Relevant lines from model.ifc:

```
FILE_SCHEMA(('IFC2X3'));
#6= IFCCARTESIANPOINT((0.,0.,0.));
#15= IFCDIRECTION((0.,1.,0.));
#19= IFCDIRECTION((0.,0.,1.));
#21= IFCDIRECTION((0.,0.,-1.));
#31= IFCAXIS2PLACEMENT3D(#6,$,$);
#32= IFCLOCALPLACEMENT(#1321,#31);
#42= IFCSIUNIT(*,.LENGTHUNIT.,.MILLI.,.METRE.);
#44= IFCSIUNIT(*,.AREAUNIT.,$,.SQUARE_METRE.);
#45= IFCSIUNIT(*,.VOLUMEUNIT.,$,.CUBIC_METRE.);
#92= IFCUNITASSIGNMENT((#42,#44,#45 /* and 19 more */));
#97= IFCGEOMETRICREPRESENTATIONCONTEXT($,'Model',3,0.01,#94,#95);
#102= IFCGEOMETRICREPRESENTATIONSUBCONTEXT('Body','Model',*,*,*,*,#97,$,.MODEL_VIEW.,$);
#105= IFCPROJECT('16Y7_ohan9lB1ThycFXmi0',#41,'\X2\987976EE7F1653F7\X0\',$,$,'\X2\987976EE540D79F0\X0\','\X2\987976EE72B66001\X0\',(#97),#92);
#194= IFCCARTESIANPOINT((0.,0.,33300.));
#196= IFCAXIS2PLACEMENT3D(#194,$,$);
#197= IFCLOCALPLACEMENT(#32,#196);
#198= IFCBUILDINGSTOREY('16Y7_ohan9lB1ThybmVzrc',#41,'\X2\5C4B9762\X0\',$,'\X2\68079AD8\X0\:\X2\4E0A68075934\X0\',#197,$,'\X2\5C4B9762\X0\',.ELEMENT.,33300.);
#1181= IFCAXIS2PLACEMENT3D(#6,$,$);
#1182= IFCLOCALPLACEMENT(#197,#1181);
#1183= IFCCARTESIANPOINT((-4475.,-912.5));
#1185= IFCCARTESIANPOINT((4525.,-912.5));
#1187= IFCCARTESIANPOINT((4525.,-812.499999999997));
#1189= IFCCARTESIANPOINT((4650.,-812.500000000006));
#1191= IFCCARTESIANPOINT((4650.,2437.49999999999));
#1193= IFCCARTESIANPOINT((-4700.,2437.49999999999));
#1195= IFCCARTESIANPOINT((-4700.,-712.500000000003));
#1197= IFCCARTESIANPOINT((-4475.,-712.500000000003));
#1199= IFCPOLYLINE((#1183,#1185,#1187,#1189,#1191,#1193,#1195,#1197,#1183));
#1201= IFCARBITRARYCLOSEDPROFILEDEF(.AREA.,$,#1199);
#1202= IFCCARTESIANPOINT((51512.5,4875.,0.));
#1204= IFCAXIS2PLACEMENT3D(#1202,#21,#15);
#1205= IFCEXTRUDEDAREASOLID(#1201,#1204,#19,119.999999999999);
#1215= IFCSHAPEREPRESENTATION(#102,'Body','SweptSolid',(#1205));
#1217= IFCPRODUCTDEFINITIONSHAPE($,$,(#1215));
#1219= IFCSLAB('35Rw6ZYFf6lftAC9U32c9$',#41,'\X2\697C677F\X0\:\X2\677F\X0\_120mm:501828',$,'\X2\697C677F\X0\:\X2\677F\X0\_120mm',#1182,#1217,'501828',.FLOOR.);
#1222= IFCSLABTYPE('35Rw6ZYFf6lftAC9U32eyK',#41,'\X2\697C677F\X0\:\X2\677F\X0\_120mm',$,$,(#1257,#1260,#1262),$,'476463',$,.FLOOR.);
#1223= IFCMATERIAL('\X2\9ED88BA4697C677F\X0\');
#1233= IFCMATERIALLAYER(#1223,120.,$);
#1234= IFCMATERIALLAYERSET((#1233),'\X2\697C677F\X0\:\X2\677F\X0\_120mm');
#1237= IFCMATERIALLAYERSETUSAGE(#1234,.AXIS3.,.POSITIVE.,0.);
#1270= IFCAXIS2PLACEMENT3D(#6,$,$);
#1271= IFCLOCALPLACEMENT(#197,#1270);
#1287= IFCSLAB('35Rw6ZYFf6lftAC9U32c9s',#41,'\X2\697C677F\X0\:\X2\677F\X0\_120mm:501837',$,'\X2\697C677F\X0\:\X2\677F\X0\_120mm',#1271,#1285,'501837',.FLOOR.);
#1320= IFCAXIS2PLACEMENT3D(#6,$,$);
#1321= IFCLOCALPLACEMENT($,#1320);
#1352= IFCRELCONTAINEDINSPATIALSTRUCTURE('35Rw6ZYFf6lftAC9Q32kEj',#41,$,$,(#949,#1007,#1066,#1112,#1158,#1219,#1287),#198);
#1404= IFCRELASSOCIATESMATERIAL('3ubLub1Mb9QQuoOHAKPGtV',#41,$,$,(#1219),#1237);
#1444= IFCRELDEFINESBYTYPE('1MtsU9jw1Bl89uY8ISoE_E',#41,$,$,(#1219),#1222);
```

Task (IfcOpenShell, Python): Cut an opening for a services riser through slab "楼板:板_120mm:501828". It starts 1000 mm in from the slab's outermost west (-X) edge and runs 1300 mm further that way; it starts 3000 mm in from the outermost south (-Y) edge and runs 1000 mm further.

```python
import numpy as np
import ifcopenshell
import ifcopenshell.api.feature
import ifcopenshell.api.geometry
import ifcopenshell.api.root
import ifcopenshell.geom
import ifcopenshell.util.placement
import ifcopenshell.util.representation
import ifcopenshell.util.shape
import ifcopenshell.util.unit

model = ifcopenshell.open("model.ifc")
unit_scale = ifcopenshell.util.unit.calculate_unit_scale(model)
settings = ifcopenshell.geom.settings()


def volume(element):
    """Net volume in cubic metres, openings subtracted."""
    shape = ifcopenshell.geom.create_shape(settings, element)
    return ifcopenshell.util.shape.get_volume(shape.geometry)


slab = model.by_guid("35Rw6ZYFf6lftAC9U32c9$")
before = volume(slab)

# Extent in the slab's own axes, in metres. The edges named are its -X and -Y sides.
slab_shape = ifcopenshell.geom.create_shape(settings, slab)
vertices = ifcopenshell.util.shape.get_vertices(slab_shape.geometry)
x_min, y_min, bottom = vertices.min(axis=0)
top = vertices[:, 2].max()

opening = ifcopenshell.api.root.create_entity(model, ifc_class="IfcOpeningElement", name="Services riser opening")
context = ifcopenshell.util.representation.get_context(model, "Model", "Body", "MODEL_VIEW")
width, depth = 1.3, 1
outline = [(0.0, 0.0), (width, 0.0), (width, depth), (0.0, depth), (0.0, 0.0)]
# Overshoot both faces by 50 mm so the cut is clean.
shape = ifcopenshell.api.geometry.add_slab_representation(
    model, context=context, depth=top - bottom + 0.1, polyline=outline
)
ifcopenshell.api.geometry.assign_representation(model, product=opening, representation=shape)

matrix = ifcopenshell.util.placement.get_local_placement(slab.ObjectPlacement)
matrix[:, 3] = matrix @ np.append(np.array([x_min + 1, y_min + 3, bottom - 0.05]) / unit_scale, 1.0)
ifcopenshell.api.geometry.edit_object_placement(model, product=opening, matrix=matrix, is_si=False)
ifcopenshell.api.feature.add_feature(model, feature=opening, element=slab)

after = volume(slab)

print(f"slab volume {before:.3f} -> {after:.3f} m3")

model.write("model-out.ifc")
```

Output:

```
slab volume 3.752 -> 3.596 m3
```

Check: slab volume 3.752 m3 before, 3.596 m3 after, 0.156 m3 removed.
